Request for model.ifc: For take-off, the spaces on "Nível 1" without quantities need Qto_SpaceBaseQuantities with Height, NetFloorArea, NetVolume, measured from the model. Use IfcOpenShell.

First a look at what the model holds.

```python
import ifcopenshell
import ifcopenshell.util.element
import ifcopenshell.util.unit

model = ifcopenshell.open("model.ifc")
print(model.schema)
for unit_type in ("LENGTHUNIT", "AREAUNIT", "VOLUMEUNIT"):
    print(unit_type, ifcopenshell.util.unit.calculate_unit_scale(model, unit_type))
storey = next(s for s in model.by_type("IfcBuildingStorey") if s.Name == "Nível 1")
spaces = [e for e in ifcopenshell.util.element.get_decomposition(storey) if e.is_a("IfcSpace")]
for e in sorted(spaces, key=lambda e: e.id()):
    print(e.id(), e.is_a(), e.Name, list(ifcopenshell.util.element.get_psets(e, qtos_only=True)), sep=" | ")
```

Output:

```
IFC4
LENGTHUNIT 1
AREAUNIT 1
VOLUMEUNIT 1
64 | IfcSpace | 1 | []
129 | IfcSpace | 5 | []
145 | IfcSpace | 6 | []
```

```python
import ifcopenshell
import ifcopenshell.api.pset
import ifcopenshell.geom
import ifcopenshell.util.element
import ifcopenshell.util.shape
import ifcopenshell.util.unit

model = ifcopenshell.open("model.ifc")
unit_scale = ifcopenshell.util.unit.calculate_unit_scale(model)
area_scale = ifcopenshell.util.unit.calculate_unit_scale(model, "AREAUNIT")
volume_scale = ifcopenshell.util.unit.calculate_unit_scale(model, "VOLUMEUNIT")
settings = ifcopenshell.geom.settings()

storey = next(s for s in model.by_type("IfcBuildingStorey") if s.Name == "Nível 1")
spaces = [e for e in ifcopenshell.util.element.get_decomposition(storey) if e.is_a("IfcSpace")]

for e in sorted(spaces, key=lambda e: e.id()):
    if ifcopenshell.util.element.get_psets(e, qtos_only=True, should_inherit=False):
        continue
    # Geometry comes back in metres, in the element's own axes.
    shape = ifcopenshell.geom.create_shape(settings, e)
    values = {
        "Height": ifcopenshell.util.shape.get_z(shape.geometry) / unit_scale,
        "NetFloorArea": ifcopenshell.util.shape.get_footprint_area(shape.geometry) / area_scale,
        "NetVolume": ifcopenshell.util.shape.get_volume(shape.geometry) / volume_scale,
    }
    qto = ifcopenshell.api.pset.add_qto(model, product=e, name="Qto_SpaceBaseQuantities")
    ifcopenshell.api.pset.edit_qto(model, qto=qto, properties=values)
    print(e.id(), {k: round(v, 3) for k, v in values.items()})

model.write("model-out.ifc")
```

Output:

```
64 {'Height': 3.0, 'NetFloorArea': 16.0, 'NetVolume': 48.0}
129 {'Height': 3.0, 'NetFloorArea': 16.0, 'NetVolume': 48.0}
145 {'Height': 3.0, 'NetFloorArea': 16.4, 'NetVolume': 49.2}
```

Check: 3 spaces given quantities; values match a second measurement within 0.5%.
